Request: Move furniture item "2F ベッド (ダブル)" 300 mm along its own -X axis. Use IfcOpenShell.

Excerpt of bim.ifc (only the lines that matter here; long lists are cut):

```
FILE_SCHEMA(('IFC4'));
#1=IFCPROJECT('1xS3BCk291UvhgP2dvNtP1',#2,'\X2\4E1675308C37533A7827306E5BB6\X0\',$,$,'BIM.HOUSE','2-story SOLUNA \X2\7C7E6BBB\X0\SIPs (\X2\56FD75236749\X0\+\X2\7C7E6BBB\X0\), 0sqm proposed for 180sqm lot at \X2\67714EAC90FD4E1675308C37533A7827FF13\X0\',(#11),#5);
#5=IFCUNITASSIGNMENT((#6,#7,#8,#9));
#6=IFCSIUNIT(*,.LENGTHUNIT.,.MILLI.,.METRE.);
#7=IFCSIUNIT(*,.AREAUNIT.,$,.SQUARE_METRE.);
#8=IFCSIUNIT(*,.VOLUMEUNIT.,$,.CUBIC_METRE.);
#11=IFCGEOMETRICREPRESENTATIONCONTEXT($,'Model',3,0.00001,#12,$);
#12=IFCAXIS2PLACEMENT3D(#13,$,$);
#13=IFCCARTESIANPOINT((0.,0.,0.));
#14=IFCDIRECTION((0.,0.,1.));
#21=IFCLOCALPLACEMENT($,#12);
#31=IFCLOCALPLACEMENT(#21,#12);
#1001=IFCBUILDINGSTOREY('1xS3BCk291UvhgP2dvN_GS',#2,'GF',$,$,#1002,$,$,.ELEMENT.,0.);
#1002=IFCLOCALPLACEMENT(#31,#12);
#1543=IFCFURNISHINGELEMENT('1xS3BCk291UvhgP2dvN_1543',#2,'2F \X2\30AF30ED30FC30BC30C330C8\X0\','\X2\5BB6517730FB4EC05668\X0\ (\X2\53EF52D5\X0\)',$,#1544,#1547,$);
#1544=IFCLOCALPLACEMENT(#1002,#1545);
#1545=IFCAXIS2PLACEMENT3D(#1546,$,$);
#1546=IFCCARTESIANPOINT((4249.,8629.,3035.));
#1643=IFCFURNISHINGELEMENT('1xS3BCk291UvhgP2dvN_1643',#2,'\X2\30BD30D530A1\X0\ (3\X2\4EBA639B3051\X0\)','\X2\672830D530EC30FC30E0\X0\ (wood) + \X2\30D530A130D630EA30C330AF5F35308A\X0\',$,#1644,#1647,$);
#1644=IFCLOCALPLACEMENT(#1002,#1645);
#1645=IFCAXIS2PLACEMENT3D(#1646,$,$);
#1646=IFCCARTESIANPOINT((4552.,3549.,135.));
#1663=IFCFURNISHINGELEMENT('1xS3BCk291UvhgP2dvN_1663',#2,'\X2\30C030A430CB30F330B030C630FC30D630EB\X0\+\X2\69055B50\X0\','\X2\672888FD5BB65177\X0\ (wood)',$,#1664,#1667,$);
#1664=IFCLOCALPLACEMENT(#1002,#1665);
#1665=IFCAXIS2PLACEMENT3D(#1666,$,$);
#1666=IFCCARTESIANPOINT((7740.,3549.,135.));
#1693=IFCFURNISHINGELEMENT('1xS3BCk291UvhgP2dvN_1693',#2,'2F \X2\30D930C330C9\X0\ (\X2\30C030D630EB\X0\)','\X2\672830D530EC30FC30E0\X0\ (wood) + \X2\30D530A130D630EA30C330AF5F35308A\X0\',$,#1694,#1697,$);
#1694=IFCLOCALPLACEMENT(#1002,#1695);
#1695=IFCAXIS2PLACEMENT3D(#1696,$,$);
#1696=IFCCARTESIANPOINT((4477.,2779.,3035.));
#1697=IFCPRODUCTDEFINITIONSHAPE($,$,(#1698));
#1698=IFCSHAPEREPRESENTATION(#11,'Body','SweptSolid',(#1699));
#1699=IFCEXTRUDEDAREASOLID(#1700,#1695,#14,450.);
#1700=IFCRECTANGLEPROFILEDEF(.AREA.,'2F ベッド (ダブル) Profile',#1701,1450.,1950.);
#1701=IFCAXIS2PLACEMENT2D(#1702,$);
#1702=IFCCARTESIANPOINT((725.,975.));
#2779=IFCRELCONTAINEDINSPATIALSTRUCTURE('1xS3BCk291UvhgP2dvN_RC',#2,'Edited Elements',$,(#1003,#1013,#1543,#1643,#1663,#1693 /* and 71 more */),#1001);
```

```python
import ifcopenshell
import ifcopenshell.api.geometry
import ifcopenshell.util.placement
import ifcopenshell.util.unit

model = ifcopenshell.open("bim.ifc")
unit_scale = ifcopenshell.util.unit.calculate_unit_scale(model)

item = model.by_guid("1xS3BCk291UvhgP2dvN_1693")
matrix = ifcopenshell.util.placement.get_local_placement(item.ObjectPlacement)
matrix[:3, 3] -= matrix[:3, 0] * 0.3 / unit_scale
ifcopenshell.api.geometry.edit_object_placement(model, product=item, matrix=matrix, is_si=False)

print(ifcopenshell.util.placement.get_local_placement(item.ObjectPlacement).round(3) + 0.0)

model.write("bim_edited.ifc")
```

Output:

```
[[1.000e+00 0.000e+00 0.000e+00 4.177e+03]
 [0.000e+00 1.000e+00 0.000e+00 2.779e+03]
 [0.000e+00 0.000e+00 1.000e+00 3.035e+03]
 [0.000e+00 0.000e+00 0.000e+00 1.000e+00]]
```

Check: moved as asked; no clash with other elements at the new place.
